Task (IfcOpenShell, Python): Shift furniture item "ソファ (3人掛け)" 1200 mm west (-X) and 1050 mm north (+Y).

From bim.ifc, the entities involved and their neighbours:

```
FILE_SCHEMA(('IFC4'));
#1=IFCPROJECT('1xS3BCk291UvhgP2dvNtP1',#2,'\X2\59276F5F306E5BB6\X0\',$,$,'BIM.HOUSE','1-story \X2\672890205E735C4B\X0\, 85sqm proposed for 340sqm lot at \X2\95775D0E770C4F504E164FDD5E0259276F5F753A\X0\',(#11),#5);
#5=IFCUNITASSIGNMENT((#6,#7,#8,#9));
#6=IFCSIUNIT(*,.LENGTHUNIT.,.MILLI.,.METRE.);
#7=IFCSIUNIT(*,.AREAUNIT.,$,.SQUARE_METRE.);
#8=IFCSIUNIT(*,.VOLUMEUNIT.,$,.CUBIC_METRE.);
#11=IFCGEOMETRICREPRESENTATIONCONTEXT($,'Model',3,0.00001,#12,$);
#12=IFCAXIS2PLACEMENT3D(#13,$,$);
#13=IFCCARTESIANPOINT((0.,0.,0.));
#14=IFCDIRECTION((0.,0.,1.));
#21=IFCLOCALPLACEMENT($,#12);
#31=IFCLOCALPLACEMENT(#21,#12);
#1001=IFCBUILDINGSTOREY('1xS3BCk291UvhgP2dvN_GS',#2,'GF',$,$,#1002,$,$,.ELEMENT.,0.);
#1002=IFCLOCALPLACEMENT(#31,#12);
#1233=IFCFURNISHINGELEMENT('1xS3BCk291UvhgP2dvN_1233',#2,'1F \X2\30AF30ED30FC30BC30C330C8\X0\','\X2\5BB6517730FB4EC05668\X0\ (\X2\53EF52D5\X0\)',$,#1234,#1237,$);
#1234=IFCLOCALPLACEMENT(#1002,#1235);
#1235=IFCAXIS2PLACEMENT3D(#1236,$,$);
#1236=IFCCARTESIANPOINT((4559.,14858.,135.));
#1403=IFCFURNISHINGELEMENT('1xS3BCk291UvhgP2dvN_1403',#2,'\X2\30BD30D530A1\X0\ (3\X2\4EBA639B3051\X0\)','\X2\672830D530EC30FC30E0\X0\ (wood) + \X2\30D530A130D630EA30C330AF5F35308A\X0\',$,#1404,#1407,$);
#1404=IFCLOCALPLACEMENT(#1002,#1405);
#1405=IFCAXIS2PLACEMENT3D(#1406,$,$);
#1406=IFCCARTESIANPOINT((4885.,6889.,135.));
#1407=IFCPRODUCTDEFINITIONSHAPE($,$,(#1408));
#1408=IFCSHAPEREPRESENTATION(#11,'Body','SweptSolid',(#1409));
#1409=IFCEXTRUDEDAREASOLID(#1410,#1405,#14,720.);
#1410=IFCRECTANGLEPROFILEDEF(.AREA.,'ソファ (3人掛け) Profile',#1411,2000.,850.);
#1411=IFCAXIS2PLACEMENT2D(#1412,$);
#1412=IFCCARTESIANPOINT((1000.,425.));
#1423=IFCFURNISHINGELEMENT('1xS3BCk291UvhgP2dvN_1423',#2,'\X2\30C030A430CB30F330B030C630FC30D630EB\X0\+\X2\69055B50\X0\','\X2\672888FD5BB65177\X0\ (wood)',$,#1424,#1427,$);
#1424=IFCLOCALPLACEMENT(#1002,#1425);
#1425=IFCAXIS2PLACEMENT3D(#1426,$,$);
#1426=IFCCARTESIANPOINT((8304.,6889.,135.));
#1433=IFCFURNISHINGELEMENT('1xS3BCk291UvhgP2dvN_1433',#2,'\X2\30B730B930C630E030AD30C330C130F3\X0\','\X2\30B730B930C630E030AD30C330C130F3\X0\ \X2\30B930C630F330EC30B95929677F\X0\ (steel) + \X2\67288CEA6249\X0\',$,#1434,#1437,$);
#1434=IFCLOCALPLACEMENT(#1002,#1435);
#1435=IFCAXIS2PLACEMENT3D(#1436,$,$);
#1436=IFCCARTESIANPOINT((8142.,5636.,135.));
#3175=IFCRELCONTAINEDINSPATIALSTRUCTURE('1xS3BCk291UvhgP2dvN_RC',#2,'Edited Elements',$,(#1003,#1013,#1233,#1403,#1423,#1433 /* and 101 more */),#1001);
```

```python
import ifcopenshell
import ifcopenshell.api.geometry
import ifcopenshell.util.placement
import ifcopenshell.util.unit

model = ifcopenshell.open("bim.ifc")
unit_scale = ifcopenshell.util.unit.calculate_unit_scale(model)

item = model.by_id(1403)
matrix = ifcopenshell.util.placement.get_local_placement(item.ObjectPlacement)
matrix[0, 3] -= 1.2 / unit_scale
matrix[1, 3] += 1.05 / unit_scale
ifcopenshell.api.geometry.edit_object_placement(model, product=item, matrix=matrix, is_si=False)

print(ifcopenshell.util.placement.get_local_placement(item.ObjectPlacement).round(3) + 0.0)

model.write("bim-out.ifc")
```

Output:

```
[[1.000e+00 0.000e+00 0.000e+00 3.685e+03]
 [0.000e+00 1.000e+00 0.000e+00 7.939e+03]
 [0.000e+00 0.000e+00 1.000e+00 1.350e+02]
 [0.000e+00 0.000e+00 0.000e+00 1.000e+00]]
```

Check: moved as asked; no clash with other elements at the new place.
